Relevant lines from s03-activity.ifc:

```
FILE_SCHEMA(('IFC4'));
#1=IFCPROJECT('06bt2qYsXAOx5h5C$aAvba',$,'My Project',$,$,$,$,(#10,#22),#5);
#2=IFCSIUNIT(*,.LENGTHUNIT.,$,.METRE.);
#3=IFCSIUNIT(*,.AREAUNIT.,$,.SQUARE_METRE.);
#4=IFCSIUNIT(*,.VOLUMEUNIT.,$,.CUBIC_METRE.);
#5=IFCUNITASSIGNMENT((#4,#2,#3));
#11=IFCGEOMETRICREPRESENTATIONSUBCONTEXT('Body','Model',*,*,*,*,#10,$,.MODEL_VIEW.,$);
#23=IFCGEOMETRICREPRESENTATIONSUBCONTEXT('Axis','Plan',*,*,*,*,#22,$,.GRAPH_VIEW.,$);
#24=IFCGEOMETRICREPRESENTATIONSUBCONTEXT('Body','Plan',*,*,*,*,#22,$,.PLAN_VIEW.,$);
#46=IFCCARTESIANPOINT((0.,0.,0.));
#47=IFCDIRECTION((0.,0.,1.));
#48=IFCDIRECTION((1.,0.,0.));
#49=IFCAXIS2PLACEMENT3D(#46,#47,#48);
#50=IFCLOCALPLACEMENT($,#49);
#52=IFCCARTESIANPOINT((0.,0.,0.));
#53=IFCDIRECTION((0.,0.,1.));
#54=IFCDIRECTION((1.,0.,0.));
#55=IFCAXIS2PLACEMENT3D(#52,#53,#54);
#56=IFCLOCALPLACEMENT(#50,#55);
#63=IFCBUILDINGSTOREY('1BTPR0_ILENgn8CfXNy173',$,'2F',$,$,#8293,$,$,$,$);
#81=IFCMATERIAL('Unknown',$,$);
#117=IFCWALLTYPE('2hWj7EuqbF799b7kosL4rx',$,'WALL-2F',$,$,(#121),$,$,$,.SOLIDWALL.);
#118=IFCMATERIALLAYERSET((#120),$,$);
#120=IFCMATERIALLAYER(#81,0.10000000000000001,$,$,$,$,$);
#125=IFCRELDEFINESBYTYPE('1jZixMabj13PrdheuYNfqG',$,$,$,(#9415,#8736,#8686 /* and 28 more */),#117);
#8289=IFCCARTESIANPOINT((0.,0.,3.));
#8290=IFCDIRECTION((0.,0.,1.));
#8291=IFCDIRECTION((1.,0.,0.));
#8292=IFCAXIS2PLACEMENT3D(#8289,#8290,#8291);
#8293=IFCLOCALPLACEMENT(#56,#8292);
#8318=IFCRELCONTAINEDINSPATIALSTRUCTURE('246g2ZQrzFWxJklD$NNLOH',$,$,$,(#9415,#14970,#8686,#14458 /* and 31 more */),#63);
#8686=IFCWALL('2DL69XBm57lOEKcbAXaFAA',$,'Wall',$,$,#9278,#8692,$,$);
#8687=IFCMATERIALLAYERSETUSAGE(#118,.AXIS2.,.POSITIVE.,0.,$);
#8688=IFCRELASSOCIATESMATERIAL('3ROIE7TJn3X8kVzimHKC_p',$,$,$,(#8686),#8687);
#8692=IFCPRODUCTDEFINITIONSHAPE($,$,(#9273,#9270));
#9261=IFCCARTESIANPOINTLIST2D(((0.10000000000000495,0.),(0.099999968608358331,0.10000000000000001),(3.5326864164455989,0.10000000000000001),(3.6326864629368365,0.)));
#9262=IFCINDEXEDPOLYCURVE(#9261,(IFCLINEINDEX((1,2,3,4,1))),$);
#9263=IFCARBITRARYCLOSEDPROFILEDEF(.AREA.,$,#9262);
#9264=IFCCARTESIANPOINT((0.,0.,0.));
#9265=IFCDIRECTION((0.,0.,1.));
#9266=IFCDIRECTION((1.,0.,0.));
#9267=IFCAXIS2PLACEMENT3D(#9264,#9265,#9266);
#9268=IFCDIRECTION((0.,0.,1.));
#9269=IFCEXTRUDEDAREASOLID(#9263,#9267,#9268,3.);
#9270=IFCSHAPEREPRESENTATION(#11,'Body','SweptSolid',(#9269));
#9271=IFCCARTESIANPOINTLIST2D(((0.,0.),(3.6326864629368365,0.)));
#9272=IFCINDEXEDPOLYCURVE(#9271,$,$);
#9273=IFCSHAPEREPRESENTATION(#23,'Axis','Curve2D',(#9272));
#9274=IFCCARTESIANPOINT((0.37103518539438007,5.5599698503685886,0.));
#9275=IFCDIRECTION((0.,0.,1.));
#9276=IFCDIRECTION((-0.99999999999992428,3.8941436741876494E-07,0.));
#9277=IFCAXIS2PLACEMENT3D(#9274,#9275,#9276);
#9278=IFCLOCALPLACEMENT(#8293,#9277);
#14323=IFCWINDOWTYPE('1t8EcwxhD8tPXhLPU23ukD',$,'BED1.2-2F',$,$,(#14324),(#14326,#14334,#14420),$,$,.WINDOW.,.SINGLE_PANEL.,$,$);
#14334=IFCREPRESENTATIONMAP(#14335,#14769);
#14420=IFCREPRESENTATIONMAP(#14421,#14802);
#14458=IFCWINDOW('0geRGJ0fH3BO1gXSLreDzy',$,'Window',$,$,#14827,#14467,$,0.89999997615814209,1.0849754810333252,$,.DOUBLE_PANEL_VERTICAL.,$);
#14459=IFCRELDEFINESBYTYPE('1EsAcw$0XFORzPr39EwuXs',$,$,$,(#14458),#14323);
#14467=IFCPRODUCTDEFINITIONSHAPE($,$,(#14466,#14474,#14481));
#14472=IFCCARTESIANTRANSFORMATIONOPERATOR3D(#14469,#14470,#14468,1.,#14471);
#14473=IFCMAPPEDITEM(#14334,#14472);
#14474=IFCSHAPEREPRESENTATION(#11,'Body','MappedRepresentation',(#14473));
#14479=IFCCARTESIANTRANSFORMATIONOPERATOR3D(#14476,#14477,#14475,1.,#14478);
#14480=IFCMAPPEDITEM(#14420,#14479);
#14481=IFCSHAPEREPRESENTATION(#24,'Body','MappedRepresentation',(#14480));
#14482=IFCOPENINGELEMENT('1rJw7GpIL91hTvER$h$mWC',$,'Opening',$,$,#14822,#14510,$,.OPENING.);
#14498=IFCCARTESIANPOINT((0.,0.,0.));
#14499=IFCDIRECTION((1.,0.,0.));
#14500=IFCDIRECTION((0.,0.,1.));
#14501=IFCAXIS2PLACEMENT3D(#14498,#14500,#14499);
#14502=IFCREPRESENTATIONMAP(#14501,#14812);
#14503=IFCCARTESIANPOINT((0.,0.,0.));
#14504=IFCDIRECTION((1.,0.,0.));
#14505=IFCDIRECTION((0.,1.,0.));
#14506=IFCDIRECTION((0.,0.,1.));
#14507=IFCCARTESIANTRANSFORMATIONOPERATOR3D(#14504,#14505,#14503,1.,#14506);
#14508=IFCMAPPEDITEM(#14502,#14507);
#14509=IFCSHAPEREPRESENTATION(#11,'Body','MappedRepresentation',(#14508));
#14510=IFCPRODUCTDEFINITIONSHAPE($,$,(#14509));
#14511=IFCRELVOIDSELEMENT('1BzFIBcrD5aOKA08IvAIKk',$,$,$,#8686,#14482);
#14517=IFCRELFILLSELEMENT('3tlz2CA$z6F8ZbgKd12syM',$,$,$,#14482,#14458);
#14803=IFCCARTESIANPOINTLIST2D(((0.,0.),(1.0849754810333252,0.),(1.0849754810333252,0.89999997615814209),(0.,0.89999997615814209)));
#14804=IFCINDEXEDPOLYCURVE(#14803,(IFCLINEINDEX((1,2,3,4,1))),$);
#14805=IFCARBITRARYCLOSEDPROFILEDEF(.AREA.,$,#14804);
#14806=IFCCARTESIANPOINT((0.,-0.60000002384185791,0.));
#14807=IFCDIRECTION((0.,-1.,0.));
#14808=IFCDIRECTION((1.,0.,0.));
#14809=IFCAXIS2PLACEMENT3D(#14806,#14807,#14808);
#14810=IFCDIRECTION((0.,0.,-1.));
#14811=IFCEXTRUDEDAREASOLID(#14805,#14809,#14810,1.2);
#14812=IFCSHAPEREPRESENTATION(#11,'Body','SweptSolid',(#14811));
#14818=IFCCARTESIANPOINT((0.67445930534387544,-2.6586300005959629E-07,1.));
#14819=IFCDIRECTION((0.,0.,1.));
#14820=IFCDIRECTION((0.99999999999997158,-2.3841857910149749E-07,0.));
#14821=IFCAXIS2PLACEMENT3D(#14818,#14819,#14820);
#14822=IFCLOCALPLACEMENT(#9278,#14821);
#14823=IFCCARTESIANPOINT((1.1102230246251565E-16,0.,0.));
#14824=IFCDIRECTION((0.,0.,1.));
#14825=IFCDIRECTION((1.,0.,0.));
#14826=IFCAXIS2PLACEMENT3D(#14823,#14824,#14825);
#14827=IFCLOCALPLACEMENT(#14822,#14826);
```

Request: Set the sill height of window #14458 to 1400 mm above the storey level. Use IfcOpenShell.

```python
import numpy as np
import ifcopenshell
import ifcopenshell.api.geometry
import ifcopenshell.geom
import ifcopenshell.util.element
import ifcopenshell.util.placement
import ifcopenshell.util.shape
import ifcopenshell.util.unit

model = ifcopenshell.open("s03-activity.ifc")
unit_scale = ifcopenshell.util.unit.calculate_unit_scale(model)

window = model.by_guid("0geRGJ0fH3BO1gXSLreDzy")
opening = window.FillsVoids[0].RelatingOpeningElement
storey = ifcopenshell.util.element.get_container(window, ifc_class="IfcBuildingStorey")
level = ifcopenshell.util.placement.get_local_placement(storey.ObjectPlacement)[2, 3]

# The opening's origin need not be at the sill, so measure its lowest point.
shape = ifcopenshell.geom.create_shape(ifcopenshell.geom.settings(), opening)
bottom = ifcopenshell.util.shape.get_shape_bottom_elevation(shape, shape.geometry) / unit_scale
dz = level + 1.4 / unit_scale - bottom

shift = np.array([0.0, 0.0, dz])
# The window is placed relative to its opening, so it follows when the opening moves.
matrix = ifcopenshell.util.placement.get_local_placement(opening.ObjectPlacement)
matrix[:3, 3] += shift
ifcopenshell.api.geometry.edit_object_placement(
    model, product=opening, matrix=matrix, is_si=False, should_transform_children=True
)

print(f"moved by {dz * unit_scale:+.3f} m")

model.write("s03-activity_edited.ifc")
```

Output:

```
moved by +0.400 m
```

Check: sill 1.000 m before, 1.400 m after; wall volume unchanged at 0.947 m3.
